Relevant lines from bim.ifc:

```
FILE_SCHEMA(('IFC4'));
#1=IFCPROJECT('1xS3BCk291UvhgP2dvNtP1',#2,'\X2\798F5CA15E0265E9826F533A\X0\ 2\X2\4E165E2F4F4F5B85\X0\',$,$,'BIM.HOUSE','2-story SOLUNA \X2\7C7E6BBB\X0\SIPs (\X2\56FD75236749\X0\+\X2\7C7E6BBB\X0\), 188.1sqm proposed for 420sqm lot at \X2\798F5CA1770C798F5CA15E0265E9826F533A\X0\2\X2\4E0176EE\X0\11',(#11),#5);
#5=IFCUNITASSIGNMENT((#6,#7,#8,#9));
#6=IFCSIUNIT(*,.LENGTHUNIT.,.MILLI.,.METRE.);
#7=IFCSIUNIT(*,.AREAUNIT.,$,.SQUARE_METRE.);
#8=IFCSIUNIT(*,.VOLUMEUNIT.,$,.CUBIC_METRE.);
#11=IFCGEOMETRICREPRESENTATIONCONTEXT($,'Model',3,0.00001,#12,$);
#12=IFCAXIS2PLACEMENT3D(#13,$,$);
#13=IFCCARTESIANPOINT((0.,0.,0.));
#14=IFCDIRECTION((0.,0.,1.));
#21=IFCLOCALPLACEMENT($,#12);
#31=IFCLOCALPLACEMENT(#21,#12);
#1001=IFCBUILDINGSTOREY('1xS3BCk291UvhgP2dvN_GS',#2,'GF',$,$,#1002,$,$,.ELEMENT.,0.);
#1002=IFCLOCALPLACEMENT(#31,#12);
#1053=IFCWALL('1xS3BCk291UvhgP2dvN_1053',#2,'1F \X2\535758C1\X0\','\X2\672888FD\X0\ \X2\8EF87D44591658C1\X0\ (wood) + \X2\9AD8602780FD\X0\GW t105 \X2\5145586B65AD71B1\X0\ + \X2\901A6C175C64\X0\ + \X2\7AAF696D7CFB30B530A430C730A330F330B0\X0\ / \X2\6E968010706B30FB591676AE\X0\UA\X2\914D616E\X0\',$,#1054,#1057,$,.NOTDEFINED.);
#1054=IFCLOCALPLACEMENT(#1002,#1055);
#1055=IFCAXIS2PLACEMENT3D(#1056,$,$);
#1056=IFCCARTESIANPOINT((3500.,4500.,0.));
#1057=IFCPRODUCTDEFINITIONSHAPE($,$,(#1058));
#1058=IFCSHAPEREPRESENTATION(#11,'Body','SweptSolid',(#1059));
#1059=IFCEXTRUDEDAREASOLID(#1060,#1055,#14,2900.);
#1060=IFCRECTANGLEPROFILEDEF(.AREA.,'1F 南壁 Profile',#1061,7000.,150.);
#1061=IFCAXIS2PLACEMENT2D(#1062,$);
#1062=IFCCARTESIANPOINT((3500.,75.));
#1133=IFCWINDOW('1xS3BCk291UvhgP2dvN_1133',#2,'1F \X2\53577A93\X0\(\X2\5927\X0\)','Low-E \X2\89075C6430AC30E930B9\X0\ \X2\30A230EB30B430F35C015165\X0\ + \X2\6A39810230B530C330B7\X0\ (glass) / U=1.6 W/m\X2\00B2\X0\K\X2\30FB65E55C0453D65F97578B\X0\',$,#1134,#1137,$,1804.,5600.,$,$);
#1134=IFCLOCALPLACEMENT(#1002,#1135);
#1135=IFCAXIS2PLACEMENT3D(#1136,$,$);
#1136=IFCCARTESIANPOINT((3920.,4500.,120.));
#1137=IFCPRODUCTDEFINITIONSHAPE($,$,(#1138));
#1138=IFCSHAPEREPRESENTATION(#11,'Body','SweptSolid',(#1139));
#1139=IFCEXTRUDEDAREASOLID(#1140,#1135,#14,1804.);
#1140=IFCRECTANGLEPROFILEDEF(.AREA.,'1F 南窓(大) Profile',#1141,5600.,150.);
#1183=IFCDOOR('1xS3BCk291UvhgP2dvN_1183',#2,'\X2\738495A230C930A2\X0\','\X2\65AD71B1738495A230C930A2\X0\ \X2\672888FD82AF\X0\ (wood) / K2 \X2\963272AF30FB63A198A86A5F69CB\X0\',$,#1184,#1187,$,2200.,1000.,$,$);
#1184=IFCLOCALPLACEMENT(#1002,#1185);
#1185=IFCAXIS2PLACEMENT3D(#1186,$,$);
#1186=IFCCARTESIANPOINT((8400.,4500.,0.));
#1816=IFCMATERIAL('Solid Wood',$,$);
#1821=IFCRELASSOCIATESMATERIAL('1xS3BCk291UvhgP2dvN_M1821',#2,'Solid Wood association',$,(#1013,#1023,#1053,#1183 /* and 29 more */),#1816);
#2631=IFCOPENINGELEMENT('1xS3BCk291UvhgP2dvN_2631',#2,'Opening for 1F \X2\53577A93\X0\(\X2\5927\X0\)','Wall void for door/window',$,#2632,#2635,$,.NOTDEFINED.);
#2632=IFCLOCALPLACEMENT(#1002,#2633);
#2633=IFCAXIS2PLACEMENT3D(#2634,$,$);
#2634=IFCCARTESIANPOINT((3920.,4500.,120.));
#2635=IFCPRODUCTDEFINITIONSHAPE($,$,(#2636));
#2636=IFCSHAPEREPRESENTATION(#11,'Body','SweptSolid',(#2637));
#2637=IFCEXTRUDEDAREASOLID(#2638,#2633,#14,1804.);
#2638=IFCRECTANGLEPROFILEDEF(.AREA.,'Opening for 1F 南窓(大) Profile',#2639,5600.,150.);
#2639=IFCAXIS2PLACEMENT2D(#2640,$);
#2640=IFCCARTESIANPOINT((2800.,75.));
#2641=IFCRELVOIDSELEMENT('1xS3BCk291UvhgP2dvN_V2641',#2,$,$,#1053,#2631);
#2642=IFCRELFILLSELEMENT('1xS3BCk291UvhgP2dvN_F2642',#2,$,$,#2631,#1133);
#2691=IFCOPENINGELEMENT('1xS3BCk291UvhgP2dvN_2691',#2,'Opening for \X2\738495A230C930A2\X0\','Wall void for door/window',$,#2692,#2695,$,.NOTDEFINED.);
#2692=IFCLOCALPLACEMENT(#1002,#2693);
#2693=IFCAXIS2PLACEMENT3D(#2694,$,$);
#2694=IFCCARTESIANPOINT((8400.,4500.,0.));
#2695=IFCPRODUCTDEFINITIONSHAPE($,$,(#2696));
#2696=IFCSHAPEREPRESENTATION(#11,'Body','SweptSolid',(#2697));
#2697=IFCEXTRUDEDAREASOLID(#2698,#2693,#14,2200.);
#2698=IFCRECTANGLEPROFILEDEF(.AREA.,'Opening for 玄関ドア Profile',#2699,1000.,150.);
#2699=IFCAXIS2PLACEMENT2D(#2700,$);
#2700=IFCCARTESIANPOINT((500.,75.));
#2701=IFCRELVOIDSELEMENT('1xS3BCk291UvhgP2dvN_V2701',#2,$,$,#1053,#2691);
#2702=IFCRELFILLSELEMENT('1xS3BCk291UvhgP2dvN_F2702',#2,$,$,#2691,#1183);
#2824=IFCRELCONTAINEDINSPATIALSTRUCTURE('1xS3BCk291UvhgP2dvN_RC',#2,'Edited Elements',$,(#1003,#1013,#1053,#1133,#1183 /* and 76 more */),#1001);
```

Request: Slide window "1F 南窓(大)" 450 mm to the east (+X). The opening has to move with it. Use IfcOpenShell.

```python
import ifcopenshell
import ifcopenshell.api.geometry
import ifcopenshell.util.placement
import ifcopenshell.util.unit

model = ifcopenshell.open("bim.ifc")
unit_scale = ifcopenshell.util.unit.calculate_unit_scale(model)

window = model.by_id(1133)
opening = window.FillsVoids[0].RelatingOpeningElement
wall = opening.VoidsElements[0].RelatingBuildingElement

wall_matrix = ifcopenshell.util.placement.get_local_placement(wall.ObjectPlacement)
shift = wall_matrix[:3, 0] * 0.45 / unit_scale
before = ifcopenshell.util.placement.get_local_placement(window.ObjectPlacement)[:3, 3].copy()

# The window is not placed relative to its opening, so move both.
for product in (opening, window):
    matrix = ifcopenshell.util.placement.get_local_placement(product.ObjectPlacement)
    matrix[:3, 3] += shift
    ifcopenshell.api.geometry.edit_object_placement(model, product=product, matrix=matrix, is_si=False)

after = ifcopenshell.util.placement.get_local_placement(window.ObjectPlacement)[:3, 3]
print("window moved by", (after - before).round(3) + 0.0)

model.write("bim_v2.ifc")
```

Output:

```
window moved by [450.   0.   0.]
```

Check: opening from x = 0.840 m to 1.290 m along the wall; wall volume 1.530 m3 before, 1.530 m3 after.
